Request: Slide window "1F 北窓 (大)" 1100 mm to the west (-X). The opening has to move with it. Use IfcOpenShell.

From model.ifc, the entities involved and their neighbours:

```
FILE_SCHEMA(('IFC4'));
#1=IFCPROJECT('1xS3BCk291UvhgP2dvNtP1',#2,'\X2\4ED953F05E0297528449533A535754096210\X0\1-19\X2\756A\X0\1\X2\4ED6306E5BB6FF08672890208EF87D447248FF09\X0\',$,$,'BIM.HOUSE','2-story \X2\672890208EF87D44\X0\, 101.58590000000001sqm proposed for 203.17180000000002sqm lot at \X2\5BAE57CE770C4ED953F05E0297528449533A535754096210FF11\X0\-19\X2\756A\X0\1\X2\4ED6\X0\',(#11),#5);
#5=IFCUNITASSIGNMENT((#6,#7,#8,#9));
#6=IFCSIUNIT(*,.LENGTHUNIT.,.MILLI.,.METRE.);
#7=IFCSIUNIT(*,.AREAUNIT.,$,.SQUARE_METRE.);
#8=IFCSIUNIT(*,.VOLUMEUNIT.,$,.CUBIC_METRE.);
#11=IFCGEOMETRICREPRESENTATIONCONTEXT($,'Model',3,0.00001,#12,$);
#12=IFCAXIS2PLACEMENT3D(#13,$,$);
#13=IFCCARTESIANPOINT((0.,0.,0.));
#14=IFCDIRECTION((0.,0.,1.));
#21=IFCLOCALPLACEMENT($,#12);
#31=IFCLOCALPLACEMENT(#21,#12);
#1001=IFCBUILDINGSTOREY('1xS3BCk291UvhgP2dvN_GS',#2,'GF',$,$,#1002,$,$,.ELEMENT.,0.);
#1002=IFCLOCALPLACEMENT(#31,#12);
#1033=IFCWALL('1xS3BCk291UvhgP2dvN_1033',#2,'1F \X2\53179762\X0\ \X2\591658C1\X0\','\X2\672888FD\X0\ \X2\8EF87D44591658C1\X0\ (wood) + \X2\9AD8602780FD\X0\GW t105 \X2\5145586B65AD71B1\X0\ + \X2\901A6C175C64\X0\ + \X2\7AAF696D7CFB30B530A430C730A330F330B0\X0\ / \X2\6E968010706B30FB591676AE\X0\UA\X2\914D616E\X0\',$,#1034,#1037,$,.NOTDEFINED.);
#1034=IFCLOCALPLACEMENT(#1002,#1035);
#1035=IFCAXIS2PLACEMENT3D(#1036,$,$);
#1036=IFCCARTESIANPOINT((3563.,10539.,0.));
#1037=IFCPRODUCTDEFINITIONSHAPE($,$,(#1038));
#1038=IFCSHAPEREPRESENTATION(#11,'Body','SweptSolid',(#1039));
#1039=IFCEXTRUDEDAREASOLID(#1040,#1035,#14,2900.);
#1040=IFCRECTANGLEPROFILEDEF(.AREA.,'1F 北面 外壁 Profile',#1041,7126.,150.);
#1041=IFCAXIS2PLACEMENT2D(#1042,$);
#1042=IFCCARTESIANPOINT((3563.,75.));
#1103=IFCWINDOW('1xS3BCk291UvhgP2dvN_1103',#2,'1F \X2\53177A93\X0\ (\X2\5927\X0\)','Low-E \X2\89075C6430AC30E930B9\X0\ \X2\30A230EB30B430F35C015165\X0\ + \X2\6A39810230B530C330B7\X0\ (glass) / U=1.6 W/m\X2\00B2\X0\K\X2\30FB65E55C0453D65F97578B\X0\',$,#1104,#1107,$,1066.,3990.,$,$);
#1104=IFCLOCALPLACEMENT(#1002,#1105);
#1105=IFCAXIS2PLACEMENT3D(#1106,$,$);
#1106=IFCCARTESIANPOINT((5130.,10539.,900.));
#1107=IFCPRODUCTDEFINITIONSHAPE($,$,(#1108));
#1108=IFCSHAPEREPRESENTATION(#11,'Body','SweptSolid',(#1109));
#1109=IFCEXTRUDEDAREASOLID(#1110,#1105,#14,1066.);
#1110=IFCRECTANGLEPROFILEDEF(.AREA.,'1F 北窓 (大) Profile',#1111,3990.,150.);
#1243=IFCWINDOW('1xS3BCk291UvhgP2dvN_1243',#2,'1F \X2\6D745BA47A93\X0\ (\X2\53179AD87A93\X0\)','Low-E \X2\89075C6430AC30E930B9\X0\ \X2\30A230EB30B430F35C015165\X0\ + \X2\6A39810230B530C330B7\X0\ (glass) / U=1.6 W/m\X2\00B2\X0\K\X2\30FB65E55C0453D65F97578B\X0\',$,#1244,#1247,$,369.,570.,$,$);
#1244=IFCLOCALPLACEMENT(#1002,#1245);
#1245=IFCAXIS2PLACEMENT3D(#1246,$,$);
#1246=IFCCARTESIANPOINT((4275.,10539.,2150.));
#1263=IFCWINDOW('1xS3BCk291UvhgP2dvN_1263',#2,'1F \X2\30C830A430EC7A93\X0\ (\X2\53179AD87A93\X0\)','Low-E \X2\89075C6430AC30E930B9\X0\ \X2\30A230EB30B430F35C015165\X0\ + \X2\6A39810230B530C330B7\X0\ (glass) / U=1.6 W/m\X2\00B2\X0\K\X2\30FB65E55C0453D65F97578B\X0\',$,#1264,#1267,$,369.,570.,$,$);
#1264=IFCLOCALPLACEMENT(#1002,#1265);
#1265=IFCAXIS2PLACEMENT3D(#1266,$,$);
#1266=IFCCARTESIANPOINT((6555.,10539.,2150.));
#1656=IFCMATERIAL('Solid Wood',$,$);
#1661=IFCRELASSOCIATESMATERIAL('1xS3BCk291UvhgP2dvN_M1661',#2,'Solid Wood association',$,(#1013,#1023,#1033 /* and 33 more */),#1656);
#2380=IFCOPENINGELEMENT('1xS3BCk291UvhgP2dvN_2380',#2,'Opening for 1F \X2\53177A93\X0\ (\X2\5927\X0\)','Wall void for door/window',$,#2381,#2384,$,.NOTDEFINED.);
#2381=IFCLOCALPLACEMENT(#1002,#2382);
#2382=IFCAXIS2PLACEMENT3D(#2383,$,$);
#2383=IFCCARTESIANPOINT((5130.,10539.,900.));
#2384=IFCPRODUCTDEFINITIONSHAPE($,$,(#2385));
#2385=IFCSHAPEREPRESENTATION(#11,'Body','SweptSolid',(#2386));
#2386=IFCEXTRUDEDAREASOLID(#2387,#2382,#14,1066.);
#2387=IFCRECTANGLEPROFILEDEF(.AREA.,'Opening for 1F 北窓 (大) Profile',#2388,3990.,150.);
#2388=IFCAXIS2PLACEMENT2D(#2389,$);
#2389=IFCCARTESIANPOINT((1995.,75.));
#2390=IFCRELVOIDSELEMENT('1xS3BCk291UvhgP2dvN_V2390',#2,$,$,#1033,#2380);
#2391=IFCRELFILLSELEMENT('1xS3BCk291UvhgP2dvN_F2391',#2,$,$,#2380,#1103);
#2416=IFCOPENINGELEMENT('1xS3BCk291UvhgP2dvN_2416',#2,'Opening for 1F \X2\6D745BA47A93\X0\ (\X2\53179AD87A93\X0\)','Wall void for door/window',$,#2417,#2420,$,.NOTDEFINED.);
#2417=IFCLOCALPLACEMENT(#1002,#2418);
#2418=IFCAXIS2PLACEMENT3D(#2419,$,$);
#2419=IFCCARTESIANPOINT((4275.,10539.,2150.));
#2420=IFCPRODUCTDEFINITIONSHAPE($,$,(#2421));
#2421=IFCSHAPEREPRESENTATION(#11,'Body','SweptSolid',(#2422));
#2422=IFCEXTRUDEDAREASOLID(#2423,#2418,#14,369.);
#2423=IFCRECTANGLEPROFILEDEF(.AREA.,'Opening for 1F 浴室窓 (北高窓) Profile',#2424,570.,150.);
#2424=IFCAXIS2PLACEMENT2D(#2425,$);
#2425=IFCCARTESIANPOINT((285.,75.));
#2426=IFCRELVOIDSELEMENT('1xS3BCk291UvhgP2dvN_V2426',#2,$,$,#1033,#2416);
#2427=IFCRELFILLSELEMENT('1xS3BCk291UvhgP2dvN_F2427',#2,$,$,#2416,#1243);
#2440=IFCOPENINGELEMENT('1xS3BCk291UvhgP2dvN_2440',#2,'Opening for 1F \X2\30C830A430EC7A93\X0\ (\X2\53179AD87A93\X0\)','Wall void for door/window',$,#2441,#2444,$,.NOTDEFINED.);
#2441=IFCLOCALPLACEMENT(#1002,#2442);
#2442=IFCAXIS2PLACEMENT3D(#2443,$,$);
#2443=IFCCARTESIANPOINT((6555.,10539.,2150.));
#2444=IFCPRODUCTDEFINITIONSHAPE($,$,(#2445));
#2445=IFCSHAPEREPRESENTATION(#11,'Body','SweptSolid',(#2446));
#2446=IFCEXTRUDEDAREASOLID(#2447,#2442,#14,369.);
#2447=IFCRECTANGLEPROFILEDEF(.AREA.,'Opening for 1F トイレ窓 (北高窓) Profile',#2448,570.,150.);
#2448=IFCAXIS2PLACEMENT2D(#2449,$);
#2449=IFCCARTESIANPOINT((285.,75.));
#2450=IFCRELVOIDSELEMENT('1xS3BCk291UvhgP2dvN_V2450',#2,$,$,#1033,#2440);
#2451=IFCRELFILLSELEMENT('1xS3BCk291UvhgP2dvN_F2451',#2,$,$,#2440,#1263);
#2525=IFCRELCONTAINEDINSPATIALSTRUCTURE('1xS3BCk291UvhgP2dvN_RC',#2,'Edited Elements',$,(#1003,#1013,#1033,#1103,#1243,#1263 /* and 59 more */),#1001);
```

```python
import ifcopenshell
import ifcopenshell.api.geometry
import ifcopenshell.util.placement

model = ifcopenshell.open("model.ifc")

window = model.by_guid("1xS3BCk291UvhgP2dvN_1103")
opening = window.FillsVoids[0].RelatingOpeningElement
wall = opening.VoidsElements[0].RelatingBuildingElement

wall_matrix = ifcopenshell.util.placement.get_local_placement(wall.ObjectPlacement)
shift = wall_matrix[:3, 0] * -1100.0
before = ifcopenshell.util.placement.get_local_placement(window.ObjectPlacement)[:3, 3].copy()

# The window is not placed relative to its opening, so move both.
for product in (opening, window):
    matrix = ifcopenshell.util.placement.get_local_placement(product.ObjectPlacement)
    matrix[:3, 3] += shift
    ifcopenshell.api.geometry.edit_object_placement(model, product=product, matrix=matrix, is_si=False)

after = ifcopenshell.util.placement.get_local_placement(window.ObjectPlacement)[:3, 3]
print("window moved by", (after - before).round(3) + 0.0)

model.write("model_v2.ifc")
```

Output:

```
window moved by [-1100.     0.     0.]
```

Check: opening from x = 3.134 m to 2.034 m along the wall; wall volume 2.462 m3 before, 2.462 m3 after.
